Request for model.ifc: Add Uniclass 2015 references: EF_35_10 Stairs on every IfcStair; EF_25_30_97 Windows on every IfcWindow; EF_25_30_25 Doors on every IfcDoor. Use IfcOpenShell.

First a look at what the model holds.

```python
import ifcopenshell

model = ifcopenshell.open("model.ifc")
print(model.schema)
print("classifications:", [c.Name for c in model.by_type("IfcClassification")])
for ifc_class in ("IfcDoor", "IfcRoof", "IfcStair", "IfcWall", "IfcWindow"):
    print(ifc_class, len(model.by_type(ifc_class)))
```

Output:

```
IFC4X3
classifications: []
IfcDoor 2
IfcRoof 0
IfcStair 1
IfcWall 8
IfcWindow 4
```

```python
import ifcopenshell
import ifcopenshell.api.classification

model = ifcopenshell.open("model.ifc")

system = ifcopenshell.api.classification.add_classification(model, classification="Uniclass 2015")

codes = {
    "IfcStair": ("EF_35_10", "Stairs"),
    "IfcWindow": ("EF_25_30_97", "Windows"),
    "IfcDoor": ("EF_25_30_25", "Doors"),
}
for ifc_class, (code, name) in codes.items():
    products = model.by_type(ifc_class)
    ifcopenshell.api.classification.add_reference(
        model, products=products, classification=system, identification=code, name=name
    )
    print(code, len(products))

model.write("model-out.ifc")
```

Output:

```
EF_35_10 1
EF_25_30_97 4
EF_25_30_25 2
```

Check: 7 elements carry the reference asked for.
